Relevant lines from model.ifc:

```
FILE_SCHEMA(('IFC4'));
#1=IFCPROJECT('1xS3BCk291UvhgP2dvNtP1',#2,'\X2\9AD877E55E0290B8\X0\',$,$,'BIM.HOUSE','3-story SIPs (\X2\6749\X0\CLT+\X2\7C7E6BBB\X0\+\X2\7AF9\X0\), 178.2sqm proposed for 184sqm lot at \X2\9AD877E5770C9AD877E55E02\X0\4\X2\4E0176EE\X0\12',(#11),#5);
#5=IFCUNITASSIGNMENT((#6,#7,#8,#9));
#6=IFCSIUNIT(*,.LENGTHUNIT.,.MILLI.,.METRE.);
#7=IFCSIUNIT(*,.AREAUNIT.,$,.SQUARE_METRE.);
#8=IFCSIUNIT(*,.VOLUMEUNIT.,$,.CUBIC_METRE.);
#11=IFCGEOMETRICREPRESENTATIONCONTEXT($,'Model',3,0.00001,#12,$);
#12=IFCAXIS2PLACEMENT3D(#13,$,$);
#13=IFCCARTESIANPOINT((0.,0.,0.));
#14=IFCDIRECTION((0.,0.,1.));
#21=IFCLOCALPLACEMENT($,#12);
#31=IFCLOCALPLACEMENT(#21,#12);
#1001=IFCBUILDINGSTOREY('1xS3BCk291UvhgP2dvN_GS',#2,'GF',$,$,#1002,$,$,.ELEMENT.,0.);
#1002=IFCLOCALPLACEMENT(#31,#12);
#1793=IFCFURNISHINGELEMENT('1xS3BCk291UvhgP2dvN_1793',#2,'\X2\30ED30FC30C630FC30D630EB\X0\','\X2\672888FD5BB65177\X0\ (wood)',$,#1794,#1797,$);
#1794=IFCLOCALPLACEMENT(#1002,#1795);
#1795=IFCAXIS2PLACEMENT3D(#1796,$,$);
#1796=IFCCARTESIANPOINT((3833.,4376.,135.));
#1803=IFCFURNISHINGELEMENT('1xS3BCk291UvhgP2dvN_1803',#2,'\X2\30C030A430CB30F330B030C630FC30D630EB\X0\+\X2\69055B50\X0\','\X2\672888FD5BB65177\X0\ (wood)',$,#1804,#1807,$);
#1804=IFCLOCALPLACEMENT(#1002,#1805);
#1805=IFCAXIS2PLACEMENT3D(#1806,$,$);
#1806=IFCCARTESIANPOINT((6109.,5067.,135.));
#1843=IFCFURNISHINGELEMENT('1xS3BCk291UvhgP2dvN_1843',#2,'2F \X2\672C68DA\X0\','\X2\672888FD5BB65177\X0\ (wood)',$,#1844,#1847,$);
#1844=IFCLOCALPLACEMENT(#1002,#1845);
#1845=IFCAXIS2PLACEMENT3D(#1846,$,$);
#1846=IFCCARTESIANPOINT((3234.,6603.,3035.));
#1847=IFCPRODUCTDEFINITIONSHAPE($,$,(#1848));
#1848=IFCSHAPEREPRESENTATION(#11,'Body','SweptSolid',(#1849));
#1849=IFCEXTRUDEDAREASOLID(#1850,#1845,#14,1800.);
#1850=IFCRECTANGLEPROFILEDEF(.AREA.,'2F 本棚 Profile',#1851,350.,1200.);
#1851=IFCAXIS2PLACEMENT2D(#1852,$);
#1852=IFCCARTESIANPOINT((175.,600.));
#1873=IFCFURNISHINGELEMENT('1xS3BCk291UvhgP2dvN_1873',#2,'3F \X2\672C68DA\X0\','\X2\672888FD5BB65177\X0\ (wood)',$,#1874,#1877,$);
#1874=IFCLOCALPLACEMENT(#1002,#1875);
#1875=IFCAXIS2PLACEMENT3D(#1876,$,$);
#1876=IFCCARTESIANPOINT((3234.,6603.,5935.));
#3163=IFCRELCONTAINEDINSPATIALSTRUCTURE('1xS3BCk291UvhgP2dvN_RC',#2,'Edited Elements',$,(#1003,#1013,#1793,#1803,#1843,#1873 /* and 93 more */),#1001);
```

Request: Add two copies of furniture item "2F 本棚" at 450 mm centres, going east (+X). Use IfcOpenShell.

```python
import numpy as np
import ifcopenshell
import ifcopenshell.api.geometry
import ifcopenshell.api.root
import ifcopenshell.util.element
import ifcopenshell.util.placement
import ifcopenshell.util.unit

model = ifcopenshell.open("model.ifc")
unit_scale = ifcopenshell.util.unit.calculate_unit_scale(model)


def reuse_history(source, copy):
    """copy_class also copies each property set's owner history, people and application; keep the originals."""
    for rel in copy.IsDefinedBy:
        if rel.is_a("IfcRelDefinesByProperties") and (history := rel.RelatingPropertyDefinition.OwnerHistory):
            rel.RelatingPropertyDefinition.OwnerHistory = source.OwnerHistory
            ifcopenshell.util.element.remove_deep2(model, history)


source = model.by_guid("1xS3BCk291UvhgP2dvN_1843")
base = ifcopenshell.util.placement.get_local_placement(source.ObjectPlacement)
step = np.array([1.0, 0.0, 0.0]) * 0.45 / unit_scale

for i in range(1, 3):
    copy = ifcopenshell.api.root.copy_class(model, product=source)
    copy.Representation = ifcopenshell.util.element.copy_deep(
        model, source.Representation, exclude=["IfcGeometricRepresentationContext", "IfcRepresentationMap"]
    )
    reuse_history(source, copy)
    matrix = base.copy()
    matrix[:3, 3] += i * step
    print("added at", matrix[:3, 3].round(3) + 0.0)
    ifcopenshell.api.geometry.edit_object_placement(model, product=copy, matrix=matrix, is_si=False)

model.write("model-out.ifc")
```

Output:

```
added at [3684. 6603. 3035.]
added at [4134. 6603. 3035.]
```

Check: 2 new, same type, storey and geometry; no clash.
